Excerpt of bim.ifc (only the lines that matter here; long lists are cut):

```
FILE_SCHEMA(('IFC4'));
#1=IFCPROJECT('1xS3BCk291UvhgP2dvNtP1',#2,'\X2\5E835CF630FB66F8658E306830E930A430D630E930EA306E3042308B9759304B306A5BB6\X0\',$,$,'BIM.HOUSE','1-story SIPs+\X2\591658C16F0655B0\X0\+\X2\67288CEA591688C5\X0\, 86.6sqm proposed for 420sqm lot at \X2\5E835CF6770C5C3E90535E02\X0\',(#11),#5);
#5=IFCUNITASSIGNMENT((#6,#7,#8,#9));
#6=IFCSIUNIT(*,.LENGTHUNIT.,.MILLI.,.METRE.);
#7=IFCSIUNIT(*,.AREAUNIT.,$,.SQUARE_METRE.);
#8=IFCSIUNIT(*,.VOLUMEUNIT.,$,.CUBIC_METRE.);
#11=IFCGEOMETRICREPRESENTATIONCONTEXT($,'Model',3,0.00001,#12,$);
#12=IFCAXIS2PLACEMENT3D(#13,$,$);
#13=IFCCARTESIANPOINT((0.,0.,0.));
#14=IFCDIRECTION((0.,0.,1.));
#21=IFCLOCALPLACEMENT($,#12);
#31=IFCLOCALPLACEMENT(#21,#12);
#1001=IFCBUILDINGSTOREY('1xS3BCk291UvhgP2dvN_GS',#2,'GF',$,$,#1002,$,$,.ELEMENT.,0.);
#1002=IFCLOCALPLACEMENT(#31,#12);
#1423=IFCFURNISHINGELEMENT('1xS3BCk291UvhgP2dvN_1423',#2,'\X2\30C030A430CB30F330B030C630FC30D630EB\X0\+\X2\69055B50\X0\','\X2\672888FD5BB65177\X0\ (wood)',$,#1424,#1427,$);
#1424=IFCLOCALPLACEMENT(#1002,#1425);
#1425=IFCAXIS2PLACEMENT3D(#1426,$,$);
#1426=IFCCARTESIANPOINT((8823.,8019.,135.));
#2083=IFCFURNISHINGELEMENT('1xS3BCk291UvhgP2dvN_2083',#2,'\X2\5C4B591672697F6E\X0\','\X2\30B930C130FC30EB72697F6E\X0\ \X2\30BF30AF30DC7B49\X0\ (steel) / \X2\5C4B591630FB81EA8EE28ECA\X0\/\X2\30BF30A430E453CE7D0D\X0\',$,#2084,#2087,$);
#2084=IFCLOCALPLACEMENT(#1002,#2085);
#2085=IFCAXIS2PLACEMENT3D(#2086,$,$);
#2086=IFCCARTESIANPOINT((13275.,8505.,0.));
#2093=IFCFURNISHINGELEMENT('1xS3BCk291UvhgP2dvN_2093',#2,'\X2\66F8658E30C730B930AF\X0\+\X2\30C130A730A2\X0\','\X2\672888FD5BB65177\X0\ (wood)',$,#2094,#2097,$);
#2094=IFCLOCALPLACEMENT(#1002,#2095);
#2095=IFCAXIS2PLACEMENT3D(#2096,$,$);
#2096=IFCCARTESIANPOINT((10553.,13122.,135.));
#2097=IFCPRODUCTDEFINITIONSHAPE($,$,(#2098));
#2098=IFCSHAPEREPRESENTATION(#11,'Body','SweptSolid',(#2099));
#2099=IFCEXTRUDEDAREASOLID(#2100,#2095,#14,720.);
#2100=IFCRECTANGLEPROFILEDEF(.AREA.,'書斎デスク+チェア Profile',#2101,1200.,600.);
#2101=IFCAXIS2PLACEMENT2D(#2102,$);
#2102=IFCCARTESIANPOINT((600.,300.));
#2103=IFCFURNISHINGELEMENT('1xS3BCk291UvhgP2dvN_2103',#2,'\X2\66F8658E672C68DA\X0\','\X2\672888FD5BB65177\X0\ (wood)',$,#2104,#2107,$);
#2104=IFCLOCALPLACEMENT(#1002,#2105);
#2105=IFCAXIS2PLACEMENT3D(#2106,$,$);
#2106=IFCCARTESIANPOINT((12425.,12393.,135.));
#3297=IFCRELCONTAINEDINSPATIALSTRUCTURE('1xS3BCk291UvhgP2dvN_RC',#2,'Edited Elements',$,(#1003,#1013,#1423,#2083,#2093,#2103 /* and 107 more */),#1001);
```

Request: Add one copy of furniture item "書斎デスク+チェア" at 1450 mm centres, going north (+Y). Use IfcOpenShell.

```python
import numpy as np
import ifcopenshell
import ifcopenshell.api.geometry
import ifcopenshell.api.root
import ifcopenshell.util.element
import ifcopenshell.util.placement
import ifcopenshell.util.unit

model = ifcopenshell.open("bim.ifc")
unit_scale = ifcopenshell.util.unit.calculate_unit_scale(model)


def reuse_history(source, copy):
    """copy_class also copies each property set's owner history, people and application; keep the originals."""
    for rel in copy.IsDefinedBy:
        if rel.is_a("IfcRelDefinesByProperties") and (history := rel.RelatingPropertyDefinition.OwnerHistory):
            rel.RelatingPropertyDefinition.OwnerHistory = source.OwnerHistory
            ifcopenshell.util.element.remove_deep2(model, history)


source = model.by_guid("1xS3BCk291UvhgP2dvN_2093")
base = ifcopenshell.util.placement.get_local_placement(source.ObjectPlacement)
step = np.array([0.0, 1.0, 0.0]) * 1.45 / unit_scale

for i in range(1, 2):
    copy = ifcopenshell.api.root.copy_class(model, product=source)
    copy.Representation = ifcopenshell.util.element.copy_deep(
        model, source.Representation, exclude=["IfcGeometricRepresentationContext", "IfcRepresentationMap"]
    )
    reuse_history(source, copy)
    matrix = base.copy()
    matrix[:3, 3] += i * step
    print("added at", matrix[:3, 3].round(3) + 0.0)
    ifcopenshell.api.geometry.edit_object_placement(model, product=copy, matrix=matrix, is_si=False)

model.write("bim_rev.ifc")
```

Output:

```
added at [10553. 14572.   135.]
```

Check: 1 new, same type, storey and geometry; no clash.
